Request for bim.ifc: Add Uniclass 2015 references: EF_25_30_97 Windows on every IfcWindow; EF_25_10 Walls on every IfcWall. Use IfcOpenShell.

First a look at what the model holds.

```python
import ifcopenshell

model = ifcopenshell.open("bim.ifc")
print(model.schema)
print("classifications:", [c.Name for c in model.by_type("IfcClassification")])
for ifc_class in ("IfcDoor", "IfcRoof", "IfcStair", "IfcWall", "IfcWindow"):
    print(ifc_class, len(model.by_type(ifc_class)))
```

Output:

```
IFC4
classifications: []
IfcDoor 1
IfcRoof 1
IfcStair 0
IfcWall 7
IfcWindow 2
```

```python
import ifcopenshell
import ifcopenshell.api.classification

model = ifcopenshell.open("bim.ifc")

system = ifcopenshell.api.classification.add_classification(model, classification="Uniclass 2015")

codes = {
    "IfcWindow": ("EF_25_30_97", "Windows"),
    "IfcWall": ("EF_25_10", "Walls"),
}
for ifc_class, (code, name) in codes.items():
    products = model.by_type(ifc_class)
    ifcopenshell.api.classification.add_reference(
        model, products=products, classification=system, identification=code, name=name
    )
    print(code, len(products))

model.write("bim_rev.ifc")
```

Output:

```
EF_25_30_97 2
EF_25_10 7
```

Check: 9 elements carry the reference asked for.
